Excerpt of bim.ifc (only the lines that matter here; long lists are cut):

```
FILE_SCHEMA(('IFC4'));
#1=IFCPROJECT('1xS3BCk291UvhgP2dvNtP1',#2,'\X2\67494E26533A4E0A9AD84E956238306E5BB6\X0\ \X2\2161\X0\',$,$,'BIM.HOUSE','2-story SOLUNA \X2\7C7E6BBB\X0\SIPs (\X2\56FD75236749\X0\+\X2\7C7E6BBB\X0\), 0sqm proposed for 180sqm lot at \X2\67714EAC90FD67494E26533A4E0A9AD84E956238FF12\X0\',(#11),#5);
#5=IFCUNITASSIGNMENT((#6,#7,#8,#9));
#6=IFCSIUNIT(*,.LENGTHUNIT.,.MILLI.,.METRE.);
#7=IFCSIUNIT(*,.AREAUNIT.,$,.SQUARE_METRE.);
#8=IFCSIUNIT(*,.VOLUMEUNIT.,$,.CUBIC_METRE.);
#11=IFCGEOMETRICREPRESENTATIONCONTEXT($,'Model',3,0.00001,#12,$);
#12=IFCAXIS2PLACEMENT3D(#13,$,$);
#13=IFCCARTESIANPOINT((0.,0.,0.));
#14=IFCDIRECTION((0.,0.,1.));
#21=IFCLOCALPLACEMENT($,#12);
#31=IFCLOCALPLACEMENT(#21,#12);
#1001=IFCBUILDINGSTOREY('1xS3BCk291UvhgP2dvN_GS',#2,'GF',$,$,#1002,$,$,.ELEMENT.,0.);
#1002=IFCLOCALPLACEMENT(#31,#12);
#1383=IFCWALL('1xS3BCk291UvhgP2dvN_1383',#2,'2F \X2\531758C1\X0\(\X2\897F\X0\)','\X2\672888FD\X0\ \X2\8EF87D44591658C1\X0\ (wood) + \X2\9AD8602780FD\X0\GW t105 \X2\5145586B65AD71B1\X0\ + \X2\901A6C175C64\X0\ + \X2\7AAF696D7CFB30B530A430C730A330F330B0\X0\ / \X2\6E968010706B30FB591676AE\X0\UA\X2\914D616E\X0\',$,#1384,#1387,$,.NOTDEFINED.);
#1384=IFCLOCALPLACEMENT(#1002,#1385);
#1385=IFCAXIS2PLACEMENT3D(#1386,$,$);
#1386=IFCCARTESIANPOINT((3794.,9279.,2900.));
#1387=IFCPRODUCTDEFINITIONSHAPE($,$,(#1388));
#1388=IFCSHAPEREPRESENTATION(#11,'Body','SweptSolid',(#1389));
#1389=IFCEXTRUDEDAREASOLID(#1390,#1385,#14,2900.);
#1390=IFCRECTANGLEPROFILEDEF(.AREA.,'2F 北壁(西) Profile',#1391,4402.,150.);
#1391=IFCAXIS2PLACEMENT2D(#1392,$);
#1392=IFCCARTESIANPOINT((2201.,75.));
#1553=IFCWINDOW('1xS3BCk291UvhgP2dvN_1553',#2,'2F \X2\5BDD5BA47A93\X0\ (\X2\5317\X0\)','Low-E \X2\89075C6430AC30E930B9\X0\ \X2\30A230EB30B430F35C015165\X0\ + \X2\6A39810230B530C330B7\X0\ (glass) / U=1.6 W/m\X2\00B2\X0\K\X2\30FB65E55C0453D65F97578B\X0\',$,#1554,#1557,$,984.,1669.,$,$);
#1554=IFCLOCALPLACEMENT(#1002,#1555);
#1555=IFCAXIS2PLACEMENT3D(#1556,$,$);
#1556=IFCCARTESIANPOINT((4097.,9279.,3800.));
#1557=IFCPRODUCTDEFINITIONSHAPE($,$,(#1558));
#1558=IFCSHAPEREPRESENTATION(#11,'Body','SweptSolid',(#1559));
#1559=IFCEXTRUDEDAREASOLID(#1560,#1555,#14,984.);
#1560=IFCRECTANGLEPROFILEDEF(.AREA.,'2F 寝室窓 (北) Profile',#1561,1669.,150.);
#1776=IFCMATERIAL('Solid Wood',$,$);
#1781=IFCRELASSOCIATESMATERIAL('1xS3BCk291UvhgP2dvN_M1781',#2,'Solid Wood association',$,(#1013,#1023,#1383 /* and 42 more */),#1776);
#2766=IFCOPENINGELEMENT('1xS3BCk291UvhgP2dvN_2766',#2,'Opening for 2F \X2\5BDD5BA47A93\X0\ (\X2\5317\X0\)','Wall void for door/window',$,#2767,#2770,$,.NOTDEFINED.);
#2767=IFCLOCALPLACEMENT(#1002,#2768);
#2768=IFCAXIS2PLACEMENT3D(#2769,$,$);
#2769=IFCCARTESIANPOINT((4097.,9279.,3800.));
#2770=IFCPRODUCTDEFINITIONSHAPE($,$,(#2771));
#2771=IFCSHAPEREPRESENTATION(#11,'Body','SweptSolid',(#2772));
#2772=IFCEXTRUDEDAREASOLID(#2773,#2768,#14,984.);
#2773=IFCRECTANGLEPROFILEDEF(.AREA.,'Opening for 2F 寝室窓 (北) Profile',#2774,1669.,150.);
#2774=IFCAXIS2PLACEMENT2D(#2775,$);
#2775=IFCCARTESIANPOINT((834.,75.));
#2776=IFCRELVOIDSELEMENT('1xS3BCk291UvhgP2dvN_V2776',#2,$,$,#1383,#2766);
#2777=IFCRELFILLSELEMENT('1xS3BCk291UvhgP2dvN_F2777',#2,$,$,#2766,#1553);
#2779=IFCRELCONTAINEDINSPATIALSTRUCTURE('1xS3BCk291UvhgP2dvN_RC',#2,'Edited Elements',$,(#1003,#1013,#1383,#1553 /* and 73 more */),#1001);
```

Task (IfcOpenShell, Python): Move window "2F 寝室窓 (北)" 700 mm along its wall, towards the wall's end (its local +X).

```python
import ifcopenshell
import ifcopenshell.api.geometry
import ifcopenshell.util.placement
import ifcopenshell.util.unit

model = ifcopenshell.open("bim.ifc")
unit_scale = ifcopenshell.util.unit.calculate_unit_scale(model)

window = model.by_id(1553)
opening = window.FillsVoids[0].RelatingOpeningElement
wall = opening.VoidsElements[0].RelatingBuildingElement

wall_matrix = ifcopenshell.util.placement.get_local_placement(wall.ObjectPlacement)
shift = wall_matrix[:3, 0] * 0.7 / unit_scale
before = ifcopenshell.util.placement.get_local_placement(window.ObjectPlacement)[:3, 3].copy()

# The window is not placed relative to its opening, so move both.
for product in (opening, window):
    matrix = ifcopenshell.util.placement.get_local_placement(product.ObjectPlacement)
    matrix[:3, 3] += shift
    ifcopenshell.api.geometry.edit_object_placement(model, product=product, matrix=matrix, is_si=False)

after = ifcopenshell.util.placement.get_local_placement(window.ObjectPlacement)[:3, 3]
print("window moved by", (after - before).round(3) + 0.0)

model.write("bim_rev.ifc")
```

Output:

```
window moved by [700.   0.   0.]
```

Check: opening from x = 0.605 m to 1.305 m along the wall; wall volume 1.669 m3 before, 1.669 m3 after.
